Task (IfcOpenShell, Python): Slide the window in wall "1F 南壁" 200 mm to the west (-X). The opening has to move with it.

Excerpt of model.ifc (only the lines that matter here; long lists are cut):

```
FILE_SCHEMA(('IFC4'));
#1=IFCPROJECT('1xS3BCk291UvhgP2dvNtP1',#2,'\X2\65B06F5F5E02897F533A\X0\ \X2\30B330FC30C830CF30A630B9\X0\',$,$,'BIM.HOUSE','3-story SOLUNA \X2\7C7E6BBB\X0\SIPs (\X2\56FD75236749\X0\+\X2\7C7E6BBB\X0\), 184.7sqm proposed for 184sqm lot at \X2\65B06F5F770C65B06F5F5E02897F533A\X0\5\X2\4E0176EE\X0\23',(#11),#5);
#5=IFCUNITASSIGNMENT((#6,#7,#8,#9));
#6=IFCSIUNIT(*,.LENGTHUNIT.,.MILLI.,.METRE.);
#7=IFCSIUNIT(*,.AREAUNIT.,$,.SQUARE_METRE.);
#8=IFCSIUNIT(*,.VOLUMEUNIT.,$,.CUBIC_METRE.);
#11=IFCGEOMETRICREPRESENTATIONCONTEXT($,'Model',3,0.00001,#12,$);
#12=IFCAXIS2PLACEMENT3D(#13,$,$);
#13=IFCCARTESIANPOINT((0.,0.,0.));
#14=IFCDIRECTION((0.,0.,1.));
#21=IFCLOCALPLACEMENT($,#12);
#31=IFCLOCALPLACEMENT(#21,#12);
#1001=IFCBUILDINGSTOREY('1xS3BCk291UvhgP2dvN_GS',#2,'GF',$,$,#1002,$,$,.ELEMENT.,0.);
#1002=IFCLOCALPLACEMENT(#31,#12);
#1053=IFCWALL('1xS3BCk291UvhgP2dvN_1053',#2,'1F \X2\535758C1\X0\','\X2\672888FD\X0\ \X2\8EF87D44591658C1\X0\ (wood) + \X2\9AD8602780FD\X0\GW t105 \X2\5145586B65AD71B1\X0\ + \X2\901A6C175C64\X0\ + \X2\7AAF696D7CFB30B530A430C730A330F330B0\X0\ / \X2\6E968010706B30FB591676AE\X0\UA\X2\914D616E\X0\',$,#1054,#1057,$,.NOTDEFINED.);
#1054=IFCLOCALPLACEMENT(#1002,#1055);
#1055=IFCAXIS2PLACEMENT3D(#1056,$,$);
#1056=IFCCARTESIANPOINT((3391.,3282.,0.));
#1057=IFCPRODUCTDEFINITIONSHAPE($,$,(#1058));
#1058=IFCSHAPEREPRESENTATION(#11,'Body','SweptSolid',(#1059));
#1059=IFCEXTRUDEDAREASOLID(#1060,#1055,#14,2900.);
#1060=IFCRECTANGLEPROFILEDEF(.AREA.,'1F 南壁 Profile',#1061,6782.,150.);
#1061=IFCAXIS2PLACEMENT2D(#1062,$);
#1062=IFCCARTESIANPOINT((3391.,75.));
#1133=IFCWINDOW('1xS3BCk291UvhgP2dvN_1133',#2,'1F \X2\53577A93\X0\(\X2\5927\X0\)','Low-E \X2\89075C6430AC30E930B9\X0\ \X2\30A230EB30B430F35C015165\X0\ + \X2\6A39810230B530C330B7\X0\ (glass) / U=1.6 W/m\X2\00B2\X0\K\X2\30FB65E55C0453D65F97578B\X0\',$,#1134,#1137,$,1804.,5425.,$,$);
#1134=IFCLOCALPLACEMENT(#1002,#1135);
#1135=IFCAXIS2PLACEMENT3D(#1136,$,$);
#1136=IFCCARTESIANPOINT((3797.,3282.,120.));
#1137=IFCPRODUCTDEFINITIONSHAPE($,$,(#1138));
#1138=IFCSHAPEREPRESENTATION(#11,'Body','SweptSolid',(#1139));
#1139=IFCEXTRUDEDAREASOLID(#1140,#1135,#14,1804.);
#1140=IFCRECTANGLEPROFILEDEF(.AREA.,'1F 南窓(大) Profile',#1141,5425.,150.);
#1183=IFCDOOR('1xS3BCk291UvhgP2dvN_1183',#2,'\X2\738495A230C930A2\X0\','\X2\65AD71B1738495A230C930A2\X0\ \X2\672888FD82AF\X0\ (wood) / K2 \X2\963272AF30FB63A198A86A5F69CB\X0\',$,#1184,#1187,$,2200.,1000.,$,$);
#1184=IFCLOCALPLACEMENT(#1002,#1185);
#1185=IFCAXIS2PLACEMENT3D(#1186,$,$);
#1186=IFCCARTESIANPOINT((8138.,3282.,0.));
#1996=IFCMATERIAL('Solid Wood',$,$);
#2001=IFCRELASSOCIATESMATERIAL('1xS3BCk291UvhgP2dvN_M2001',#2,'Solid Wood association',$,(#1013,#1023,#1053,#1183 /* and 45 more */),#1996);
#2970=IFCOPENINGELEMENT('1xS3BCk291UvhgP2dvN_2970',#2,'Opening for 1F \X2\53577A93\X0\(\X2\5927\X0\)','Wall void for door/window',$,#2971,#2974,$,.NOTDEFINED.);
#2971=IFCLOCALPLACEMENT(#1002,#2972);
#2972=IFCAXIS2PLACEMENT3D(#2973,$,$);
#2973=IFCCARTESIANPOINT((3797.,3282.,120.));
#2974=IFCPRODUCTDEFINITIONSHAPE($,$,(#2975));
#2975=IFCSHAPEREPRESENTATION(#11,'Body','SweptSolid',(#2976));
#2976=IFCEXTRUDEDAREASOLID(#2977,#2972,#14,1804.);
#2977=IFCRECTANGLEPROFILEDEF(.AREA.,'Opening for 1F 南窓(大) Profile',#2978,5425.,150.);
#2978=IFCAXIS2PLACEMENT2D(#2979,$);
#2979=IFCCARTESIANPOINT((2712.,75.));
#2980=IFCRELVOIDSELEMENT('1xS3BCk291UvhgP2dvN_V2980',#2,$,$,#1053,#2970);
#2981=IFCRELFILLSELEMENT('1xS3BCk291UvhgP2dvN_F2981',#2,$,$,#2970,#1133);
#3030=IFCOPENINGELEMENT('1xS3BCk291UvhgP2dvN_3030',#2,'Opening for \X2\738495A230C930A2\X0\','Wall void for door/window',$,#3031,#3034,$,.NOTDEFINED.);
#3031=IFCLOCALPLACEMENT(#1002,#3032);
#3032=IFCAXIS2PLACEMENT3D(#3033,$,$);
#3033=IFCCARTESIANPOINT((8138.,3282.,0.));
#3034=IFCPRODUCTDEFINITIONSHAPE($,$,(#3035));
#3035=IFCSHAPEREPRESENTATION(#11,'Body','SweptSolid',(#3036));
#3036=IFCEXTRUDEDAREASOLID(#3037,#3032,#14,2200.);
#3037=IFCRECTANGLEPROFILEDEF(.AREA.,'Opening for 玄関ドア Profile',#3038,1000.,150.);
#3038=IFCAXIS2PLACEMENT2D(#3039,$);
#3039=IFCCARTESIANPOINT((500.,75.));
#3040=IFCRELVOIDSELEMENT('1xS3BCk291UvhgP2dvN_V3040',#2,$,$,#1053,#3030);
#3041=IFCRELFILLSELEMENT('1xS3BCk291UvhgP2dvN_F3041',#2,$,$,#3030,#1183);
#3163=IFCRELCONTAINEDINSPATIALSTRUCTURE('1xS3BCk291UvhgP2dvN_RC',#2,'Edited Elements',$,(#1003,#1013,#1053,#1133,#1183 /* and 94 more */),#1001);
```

```python
import ifcopenshell
import ifcopenshell.api.geometry
import ifcopenshell.util.placement

model = ifcopenshell.open("model.ifc")

window = model.by_guid("1xS3BCk291UvhgP2dvN_1133")
opening = window.FillsVoids[0].RelatingOpeningElement
wall = opening.VoidsElements[0].RelatingBuildingElement

wall_matrix = ifcopenshell.util.placement.get_local_placement(wall.ObjectPlacement)
shift = wall_matrix[:3, 0] * -200.0
before = ifcopenshell.util.placement.get_local_placement(window.ObjectPlacement)[:3, 3].copy()

# The window is not placed relative to its opening, so move both.
for product in (opening, window):
    matrix = ifcopenshell.util.placement.get_local_placement(product.ObjectPlacement)
    matrix[:3, 3] += shift
    ifcopenshell.api.geometry.edit_object_placement(model, product=product, matrix=matrix, is_si=False)

after = ifcopenshell.util.placement.get_local_placement(window.ObjectPlacement)[:3, 3]
print("window moved by", (after - before).round(3) + 0.0)

model.write("model_edited.ifc")
```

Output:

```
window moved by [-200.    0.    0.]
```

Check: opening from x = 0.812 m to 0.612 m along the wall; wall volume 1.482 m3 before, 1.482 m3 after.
